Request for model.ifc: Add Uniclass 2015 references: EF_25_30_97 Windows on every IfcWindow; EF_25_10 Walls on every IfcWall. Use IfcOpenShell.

First a look at what the model holds.

```python
import ifcopenshell

model = ifcopenshell.open("model.ifc")
print(model.schema)
print("classifications:", [c.Name for c in model.by_type("IfcClassification")])
for ifc_class in ("IfcDoor", "IfcRoof", "IfcStair", "IfcWall", "IfcWindow"):
    print(ifc_class, len(model.by_type(ifc_class)))
```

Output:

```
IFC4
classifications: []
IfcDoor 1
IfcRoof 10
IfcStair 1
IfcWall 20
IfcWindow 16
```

```python
import ifcopenshell
import ifcopenshell.api.classification

model = ifcopenshell.open("model.ifc")

system = ifcopenshell.api.classification.add_classification(model, classification="Uniclass 2015")

codes = {
    "IfcWindow": ("EF_25_30_97", "Windows"),
    "IfcWall": ("EF_25_10", "Walls"),
}
for ifc_class, (code, name) in codes.items():
    products = model.by_type(ifc_class)
    ifcopenshell.api.classification.add_reference(
        model, products=products, classification=system, identification=code, name=name
    )
    print(code, len(products))

model.write("model_v2.ifc")
```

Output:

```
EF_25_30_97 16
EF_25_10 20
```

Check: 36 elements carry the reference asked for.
